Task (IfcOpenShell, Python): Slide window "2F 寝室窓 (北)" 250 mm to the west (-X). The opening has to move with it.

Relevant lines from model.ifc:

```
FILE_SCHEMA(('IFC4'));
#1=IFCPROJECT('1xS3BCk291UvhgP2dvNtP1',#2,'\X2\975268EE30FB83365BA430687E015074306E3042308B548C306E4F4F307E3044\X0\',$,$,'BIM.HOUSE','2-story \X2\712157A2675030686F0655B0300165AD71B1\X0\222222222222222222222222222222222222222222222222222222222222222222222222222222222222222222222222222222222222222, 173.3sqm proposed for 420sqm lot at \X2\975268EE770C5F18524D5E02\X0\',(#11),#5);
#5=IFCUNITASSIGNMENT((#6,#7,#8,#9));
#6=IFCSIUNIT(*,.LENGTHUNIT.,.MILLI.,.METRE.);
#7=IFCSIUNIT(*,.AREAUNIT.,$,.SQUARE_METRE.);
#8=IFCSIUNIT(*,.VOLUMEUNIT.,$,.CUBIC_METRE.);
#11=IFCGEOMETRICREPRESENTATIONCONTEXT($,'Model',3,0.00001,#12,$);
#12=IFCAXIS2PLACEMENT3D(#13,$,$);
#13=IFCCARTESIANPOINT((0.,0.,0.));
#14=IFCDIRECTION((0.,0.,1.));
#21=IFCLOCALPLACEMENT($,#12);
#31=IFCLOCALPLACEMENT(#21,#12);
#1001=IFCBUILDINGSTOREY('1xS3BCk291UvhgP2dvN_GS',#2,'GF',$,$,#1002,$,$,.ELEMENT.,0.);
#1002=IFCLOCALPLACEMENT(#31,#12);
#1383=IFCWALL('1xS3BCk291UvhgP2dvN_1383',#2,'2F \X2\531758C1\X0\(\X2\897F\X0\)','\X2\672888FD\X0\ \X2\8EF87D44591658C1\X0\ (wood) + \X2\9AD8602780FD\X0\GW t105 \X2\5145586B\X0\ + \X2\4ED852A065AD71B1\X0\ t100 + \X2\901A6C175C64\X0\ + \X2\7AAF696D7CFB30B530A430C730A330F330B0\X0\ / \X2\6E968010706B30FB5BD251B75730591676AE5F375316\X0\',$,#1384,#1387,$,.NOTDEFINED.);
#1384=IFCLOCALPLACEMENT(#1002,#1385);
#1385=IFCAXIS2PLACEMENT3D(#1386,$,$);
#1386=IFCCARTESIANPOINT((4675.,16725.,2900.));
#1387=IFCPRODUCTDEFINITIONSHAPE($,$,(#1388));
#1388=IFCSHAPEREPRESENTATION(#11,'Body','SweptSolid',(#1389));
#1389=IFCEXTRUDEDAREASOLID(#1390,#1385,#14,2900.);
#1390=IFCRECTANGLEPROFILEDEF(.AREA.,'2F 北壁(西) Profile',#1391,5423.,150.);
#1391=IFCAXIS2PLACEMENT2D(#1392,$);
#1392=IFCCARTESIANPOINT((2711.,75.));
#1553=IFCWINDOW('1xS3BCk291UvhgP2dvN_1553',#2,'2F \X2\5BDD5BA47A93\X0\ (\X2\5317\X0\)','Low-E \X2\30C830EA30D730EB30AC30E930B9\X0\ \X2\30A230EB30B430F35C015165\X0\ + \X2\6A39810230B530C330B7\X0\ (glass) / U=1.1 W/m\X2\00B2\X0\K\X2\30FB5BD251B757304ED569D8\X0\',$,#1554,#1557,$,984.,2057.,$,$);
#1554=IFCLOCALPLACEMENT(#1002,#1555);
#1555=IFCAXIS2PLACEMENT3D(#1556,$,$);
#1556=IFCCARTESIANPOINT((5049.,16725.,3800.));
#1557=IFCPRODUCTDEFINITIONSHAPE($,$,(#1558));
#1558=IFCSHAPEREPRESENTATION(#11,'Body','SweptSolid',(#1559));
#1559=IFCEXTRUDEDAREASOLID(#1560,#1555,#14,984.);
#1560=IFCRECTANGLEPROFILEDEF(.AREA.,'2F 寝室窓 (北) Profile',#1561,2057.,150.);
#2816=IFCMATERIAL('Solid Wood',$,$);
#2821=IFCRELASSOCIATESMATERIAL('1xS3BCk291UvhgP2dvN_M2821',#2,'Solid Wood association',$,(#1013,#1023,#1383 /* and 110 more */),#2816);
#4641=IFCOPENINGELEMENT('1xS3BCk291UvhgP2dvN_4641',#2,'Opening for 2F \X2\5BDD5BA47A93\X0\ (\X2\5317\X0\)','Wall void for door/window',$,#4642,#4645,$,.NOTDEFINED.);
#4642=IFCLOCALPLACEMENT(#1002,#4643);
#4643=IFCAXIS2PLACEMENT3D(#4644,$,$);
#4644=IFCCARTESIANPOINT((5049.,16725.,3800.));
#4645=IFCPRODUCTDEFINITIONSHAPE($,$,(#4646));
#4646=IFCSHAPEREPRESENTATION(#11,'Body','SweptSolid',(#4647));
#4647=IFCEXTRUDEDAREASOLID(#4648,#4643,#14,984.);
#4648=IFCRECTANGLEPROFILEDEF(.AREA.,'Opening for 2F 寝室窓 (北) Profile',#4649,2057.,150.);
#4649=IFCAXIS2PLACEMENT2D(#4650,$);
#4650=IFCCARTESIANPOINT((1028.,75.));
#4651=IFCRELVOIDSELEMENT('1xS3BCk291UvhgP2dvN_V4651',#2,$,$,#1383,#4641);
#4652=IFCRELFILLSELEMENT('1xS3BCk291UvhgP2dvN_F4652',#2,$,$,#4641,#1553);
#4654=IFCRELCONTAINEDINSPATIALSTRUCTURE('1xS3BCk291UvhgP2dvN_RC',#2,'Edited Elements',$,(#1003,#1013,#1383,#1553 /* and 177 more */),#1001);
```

```python
import ifcopenshell
import ifcopenshell.api.geometry
import ifcopenshell.util.placement

model = ifcopenshell.open("model.ifc")

window = model.by_id(1553)
opening = window.FillsVoids[0].RelatingOpeningElement
wall = opening.VoidsElements[0].RelatingBuildingElement

wall_matrix = ifcopenshell.util.placement.get_local_placement(wall.ObjectPlacement)
shift = wall_matrix[:3, 0] * -250.0
before = ifcopenshell.util.placement.get_local_placement(window.ObjectPlacement)[:3, 3].copy()

# The window is not placed relative to its opening, so move both.
for product in (opening, window):
    matrix = ifcopenshell.util.placement.get_local_placement(product.ObjectPlacement)
    matrix[:3, 3] += shift
    ifcopenshell.api.geometry.edit_object_placement(model, product=product, matrix=matrix, is_si=False)

after = ifcopenshell.util.placement.get_local_placement(window.ObjectPlacement)[:3, 3]
print("window moved by", (after - before).round(3) + 0.0)

model.write("model_rev.ifc")
```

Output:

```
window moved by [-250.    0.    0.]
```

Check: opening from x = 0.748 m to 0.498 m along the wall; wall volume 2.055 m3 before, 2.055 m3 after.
